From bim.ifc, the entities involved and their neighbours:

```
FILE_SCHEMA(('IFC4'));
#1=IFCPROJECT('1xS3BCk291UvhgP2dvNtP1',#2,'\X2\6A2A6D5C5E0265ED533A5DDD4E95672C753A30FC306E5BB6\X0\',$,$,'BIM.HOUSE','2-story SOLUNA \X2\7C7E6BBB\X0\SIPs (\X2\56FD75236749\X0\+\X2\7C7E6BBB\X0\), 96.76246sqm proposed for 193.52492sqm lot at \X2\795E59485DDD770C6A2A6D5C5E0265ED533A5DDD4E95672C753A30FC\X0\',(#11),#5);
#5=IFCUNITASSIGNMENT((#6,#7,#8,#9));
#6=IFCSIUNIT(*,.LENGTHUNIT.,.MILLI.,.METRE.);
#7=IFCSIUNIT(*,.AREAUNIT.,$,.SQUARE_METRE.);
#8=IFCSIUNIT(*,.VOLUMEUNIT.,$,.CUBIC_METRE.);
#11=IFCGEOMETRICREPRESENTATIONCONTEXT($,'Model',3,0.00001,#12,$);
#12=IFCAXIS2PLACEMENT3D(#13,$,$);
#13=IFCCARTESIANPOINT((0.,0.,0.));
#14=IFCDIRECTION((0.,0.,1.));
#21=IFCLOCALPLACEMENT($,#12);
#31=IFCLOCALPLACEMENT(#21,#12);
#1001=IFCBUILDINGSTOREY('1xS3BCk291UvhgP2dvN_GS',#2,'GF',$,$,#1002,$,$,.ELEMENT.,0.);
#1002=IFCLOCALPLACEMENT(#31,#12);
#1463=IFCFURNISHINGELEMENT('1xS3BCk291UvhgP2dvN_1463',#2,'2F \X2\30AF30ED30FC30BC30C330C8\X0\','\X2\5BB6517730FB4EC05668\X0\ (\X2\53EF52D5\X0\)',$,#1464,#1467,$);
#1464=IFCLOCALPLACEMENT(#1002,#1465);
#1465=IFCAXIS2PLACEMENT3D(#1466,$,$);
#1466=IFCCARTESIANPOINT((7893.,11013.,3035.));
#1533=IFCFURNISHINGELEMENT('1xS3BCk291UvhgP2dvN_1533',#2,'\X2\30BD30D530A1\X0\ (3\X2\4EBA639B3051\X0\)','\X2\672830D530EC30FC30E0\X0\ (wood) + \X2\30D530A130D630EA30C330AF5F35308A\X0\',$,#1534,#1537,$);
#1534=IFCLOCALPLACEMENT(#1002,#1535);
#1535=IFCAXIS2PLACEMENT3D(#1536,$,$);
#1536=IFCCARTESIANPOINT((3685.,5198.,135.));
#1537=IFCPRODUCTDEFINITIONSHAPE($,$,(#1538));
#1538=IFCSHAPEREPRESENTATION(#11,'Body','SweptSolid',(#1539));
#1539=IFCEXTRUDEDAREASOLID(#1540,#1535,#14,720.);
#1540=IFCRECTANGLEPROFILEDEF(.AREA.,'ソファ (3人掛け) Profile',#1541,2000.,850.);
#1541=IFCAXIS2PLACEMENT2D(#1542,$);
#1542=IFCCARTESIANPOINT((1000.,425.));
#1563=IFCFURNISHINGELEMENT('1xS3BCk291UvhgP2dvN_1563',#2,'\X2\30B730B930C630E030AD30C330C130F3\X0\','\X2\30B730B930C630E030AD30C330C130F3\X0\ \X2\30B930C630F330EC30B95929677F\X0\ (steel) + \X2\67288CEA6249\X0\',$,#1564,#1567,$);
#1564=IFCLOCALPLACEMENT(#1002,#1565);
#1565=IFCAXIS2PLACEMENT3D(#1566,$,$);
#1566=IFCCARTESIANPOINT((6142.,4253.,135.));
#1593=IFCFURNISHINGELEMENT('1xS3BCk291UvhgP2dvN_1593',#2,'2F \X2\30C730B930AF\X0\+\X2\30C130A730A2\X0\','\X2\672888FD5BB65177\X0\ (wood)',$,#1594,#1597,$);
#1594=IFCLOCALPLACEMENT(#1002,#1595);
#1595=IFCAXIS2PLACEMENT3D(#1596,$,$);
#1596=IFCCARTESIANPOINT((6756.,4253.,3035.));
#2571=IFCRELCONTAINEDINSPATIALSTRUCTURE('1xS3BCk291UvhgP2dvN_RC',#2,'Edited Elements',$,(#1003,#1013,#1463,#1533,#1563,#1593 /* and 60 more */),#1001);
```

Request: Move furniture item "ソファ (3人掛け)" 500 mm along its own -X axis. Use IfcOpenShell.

```python
import ifcopenshell
import ifcopenshell.api.geometry
import ifcopenshell.util.placement
import ifcopenshell.util.unit

model = ifcopenshell.open("bim.ifc")
unit_scale = ifcopenshell.util.unit.calculate_unit_scale(model)

item = model.by_guid("1xS3BCk291UvhgP2dvN_1533")
matrix = ifcopenshell.util.placement.get_local_placement(item.ObjectPlacement)
matrix[:3, 3] -= matrix[:3, 0] * 0.5 / unit_scale
ifcopenshell.api.geometry.edit_object_placement(model, product=item, matrix=matrix, is_si=False)

print(ifcopenshell.util.placement.get_local_placement(item.ObjectPlacement).round(3) + 0.0)

model.write("bim-out.ifc")
```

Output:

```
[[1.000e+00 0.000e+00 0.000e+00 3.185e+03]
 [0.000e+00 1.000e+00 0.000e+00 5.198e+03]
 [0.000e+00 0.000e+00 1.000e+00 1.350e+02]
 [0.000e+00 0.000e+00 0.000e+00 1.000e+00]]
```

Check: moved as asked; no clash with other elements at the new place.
